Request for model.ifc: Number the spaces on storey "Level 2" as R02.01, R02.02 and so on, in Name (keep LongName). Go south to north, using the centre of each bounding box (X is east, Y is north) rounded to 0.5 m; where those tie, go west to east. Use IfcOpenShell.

First a look at what the model holds.

```python
import ifcopenshell
import ifcopenshell.util.element
import ifcopenshell.util.placement

model = ifcopenshell.open("model.ifc")
print(model.schema)
storey = next(s for s in model.by_type("IfcBuildingStorey") if s.Name == "Level 2")
spaces = [e for e in ifcopenshell.util.element.get_decomposition(storey) if e.is_a("IfcSpace")]
for e in sorted(spaces, key=lambda e: e.id()):
    origin = ifcopenshell.util.placement.get_local_placement(e.ObjectPlacement)[:3, 3]
    print(e.id(), e.Name, e.LongName, origin.round(2) + 0.0, sep=" | ")
```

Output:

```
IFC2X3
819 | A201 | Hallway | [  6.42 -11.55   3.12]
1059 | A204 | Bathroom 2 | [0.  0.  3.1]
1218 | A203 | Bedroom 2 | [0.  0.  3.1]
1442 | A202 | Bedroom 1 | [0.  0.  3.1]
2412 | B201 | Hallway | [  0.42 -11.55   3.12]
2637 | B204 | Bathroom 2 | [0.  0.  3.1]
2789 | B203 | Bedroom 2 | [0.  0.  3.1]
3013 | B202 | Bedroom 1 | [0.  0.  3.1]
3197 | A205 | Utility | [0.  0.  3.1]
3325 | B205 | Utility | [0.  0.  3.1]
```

```python
import ifcopenshell
import ifcopenshell.geom
import ifcopenshell.util.element
import ifcopenshell.util.shape

model = ifcopenshell.open("model.ifc")
settings = ifcopenshell.geom.settings()
settings.set("use-world-coords", True)


def centre(element):
    shape = ifcopenshell.geom.create_shape(settings, element)
    return ifcopenshell.util.shape.get_bbox_centroid(shape.geometry)


storey = next(s for s in model.by_type("IfcBuildingStorey") if s.Name == "Level 2")
spaces = [e for e in ifcopenshell.util.element.get_decomposition(storey) if e.is_a("IfcSpace")]

# Insertion points can sit at a corner or the storey origin, so sort by the geometry (in metres).
centres = {e: centre(e) for e in spaces}
spaces.sort(key=lambda e: (round(centres[e][1] / 0.5), centres[e][0]))

for i, e in enumerate(spaces, start=1):
    number = f"R02.{i:02d}"
    e.Name = number
    print(e.id(), number)

model.write("model_rev.ifc")
```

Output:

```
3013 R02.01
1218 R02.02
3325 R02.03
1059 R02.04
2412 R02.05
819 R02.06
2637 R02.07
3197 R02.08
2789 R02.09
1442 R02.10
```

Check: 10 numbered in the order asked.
